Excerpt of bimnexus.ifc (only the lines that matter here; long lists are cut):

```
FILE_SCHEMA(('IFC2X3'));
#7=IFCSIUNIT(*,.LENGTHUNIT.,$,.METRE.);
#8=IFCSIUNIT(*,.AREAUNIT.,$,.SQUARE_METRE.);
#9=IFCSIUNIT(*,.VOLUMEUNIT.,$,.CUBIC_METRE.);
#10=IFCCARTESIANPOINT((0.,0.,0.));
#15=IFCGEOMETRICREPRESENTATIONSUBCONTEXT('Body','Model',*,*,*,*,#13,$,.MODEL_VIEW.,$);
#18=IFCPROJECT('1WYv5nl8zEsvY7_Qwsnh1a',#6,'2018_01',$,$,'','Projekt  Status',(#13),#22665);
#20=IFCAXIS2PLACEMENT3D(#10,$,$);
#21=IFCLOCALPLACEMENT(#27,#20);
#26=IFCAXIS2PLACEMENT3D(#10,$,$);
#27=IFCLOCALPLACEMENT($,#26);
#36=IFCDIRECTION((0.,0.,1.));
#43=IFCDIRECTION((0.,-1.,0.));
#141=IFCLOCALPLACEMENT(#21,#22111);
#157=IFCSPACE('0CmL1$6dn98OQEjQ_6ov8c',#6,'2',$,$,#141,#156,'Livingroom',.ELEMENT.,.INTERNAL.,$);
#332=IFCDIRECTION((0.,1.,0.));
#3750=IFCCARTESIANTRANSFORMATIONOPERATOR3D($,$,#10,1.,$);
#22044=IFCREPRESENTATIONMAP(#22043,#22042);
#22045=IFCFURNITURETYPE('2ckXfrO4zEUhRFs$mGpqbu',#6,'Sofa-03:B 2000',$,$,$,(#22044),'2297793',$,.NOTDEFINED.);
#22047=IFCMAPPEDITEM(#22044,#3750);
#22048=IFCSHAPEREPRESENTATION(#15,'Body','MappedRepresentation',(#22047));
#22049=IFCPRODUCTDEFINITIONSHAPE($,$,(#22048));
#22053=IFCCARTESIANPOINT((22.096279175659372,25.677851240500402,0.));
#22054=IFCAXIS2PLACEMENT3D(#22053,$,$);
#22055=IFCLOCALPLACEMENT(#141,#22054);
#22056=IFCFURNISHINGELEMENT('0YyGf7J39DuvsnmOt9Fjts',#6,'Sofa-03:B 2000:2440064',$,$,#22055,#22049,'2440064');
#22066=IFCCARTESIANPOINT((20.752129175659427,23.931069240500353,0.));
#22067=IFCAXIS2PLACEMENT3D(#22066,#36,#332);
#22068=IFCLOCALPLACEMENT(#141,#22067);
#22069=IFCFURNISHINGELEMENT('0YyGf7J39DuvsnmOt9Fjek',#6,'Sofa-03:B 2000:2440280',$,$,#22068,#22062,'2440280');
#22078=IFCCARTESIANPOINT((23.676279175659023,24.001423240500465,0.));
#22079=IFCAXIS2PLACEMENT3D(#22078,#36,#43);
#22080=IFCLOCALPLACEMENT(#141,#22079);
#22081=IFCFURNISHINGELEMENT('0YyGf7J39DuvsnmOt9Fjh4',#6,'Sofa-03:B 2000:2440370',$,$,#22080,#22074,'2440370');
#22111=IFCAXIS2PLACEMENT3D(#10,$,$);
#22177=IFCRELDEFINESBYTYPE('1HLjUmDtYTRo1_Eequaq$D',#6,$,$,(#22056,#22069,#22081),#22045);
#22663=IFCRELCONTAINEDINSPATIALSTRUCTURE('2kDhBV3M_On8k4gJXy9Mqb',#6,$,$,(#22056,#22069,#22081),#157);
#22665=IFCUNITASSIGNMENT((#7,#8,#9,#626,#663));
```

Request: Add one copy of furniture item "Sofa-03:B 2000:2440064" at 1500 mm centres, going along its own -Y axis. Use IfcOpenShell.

```python
import ifcopenshell
import ifcopenshell.api.geometry
import ifcopenshell.api.root
import ifcopenshell.util.element
import ifcopenshell.util.placement
import ifcopenshell.util.unit

model = ifcopenshell.open("bimnexus.ifc")
unit_scale = ifcopenshell.util.unit.calculate_unit_scale(model)


def reuse_history(source, copy):
    """copy_class also copies each property set's owner history, people and application; keep the originals."""
    for rel in copy.IsDefinedBy:
        if rel.is_a("IfcRelDefinesByProperties") and (history := rel.RelatingPropertyDefinition.OwnerHistory):
            rel.RelatingPropertyDefinition.OwnerHistory = source.OwnerHistory
            ifcopenshell.util.element.remove_deep2(model, history)


source = model.by_id(22056)
base = ifcopenshell.util.placement.get_local_placement(source.ObjectPlacement)
step = -base[:3, 1] * 1.5 / unit_scale

for i in range(1, 2):
    copy = ifcopenshell.api.root.copy_class(model, product=source)
    copy.Representation = ifcopenshell.util.element.copy_deep(
        model, source.Representation, exclude=["IfcGeometricRepresentationContext", "IfcRepresentationMap"]
    )
    copy.Name = "Sofa-03:B 2000"
    copy.Tag = None
    reuse_history(source, copy)
    matrix = base.copy()
    matrix[:3, 3] += i * step
    print("added at", matrix[:3, 3].round(3) + 0.0)
    ifcopenshell.api.geometry.edit_object_placement(model, product=copy, matrix=matrix, is_si=False)

model.write("bimnexus_edited.ifc")
```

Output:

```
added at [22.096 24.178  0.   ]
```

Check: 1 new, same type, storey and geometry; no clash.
